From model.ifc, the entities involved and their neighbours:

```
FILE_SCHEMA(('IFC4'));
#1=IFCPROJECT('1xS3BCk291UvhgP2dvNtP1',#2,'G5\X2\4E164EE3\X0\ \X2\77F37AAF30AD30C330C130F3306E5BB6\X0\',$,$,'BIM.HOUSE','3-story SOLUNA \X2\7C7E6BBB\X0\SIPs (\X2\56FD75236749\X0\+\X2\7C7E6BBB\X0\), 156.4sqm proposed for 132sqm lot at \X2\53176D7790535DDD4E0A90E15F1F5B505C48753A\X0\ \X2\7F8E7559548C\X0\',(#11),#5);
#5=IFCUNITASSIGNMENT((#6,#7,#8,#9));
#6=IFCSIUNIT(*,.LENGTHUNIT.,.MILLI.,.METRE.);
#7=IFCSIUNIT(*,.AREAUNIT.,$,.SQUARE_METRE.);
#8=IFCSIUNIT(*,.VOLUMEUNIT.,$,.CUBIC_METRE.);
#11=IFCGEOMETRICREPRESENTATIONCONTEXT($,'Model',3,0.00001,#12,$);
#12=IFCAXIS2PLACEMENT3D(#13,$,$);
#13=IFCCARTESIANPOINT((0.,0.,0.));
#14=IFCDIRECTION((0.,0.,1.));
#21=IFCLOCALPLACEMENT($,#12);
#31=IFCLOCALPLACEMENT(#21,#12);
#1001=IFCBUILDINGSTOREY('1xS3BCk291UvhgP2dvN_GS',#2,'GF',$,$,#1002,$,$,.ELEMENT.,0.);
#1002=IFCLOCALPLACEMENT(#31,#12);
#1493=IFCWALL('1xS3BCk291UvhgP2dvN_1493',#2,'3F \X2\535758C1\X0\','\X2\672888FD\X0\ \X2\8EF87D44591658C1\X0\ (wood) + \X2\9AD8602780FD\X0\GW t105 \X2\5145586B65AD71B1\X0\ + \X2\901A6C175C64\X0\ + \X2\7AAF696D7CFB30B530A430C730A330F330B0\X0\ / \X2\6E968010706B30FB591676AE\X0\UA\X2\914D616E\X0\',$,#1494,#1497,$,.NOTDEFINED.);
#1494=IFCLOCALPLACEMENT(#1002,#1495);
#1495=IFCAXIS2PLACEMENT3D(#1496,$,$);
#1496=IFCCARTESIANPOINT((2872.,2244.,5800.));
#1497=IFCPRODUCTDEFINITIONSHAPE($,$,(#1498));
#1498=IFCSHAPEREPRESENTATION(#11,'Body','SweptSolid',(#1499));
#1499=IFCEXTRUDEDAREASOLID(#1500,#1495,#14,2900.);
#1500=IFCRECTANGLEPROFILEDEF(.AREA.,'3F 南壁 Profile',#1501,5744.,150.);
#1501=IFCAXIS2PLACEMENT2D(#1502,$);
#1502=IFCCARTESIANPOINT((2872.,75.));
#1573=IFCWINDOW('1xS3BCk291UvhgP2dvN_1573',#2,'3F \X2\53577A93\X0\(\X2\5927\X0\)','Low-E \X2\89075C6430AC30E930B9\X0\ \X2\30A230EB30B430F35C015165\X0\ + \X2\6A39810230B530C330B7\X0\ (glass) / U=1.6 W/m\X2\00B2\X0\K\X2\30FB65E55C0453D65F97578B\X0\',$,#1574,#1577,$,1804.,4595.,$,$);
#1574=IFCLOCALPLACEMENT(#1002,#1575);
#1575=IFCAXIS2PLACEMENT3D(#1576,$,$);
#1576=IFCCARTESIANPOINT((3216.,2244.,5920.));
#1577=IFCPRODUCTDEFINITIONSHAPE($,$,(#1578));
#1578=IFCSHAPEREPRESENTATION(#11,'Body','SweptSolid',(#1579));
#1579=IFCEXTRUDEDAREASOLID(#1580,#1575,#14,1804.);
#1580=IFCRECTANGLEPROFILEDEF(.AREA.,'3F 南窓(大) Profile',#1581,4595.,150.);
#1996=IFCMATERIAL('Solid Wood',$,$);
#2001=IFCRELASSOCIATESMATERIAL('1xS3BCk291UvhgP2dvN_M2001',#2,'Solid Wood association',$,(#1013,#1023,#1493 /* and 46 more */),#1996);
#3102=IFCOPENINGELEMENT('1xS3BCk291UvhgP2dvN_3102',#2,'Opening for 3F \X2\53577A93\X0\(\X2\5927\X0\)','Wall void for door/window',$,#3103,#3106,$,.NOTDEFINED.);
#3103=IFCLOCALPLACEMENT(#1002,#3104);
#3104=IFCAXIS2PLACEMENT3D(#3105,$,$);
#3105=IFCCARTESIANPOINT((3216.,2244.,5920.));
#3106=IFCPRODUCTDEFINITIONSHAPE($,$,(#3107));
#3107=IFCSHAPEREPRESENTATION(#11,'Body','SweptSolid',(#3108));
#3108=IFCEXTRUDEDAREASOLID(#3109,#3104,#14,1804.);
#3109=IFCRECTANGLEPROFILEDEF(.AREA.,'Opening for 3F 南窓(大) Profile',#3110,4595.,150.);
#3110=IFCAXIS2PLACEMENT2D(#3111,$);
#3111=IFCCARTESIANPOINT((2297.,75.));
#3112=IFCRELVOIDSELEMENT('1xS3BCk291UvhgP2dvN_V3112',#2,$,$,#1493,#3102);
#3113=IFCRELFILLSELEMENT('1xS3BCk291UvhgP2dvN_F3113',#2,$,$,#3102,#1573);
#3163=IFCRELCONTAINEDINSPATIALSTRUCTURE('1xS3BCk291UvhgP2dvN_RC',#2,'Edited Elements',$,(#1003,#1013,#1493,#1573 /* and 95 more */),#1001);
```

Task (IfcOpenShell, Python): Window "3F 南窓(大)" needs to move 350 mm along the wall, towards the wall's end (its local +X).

```python
import ifcopenshell
import ifcopenshell.api.geometry
import ifcopenshell.util.placement

model = ifcopenshell.open("model.ifc")

window = model.by_guid("1xS3BCk291UvhgP2dvN_1573")
opening = window.FillsVoids[0].RelatingOpeningElement
wall = opening.VoidsElements[0].RelatingBuildingElement

wall_matrix = ifcopenshell.util.placement.get_local_placement(wall.ObjectPlacement)
shift = wall_matrix[:3, 0] * 350.0
before = ifcopenshell.util.placement.get_local_placement(window.ObjectPlacement)[:3, 3].copy()

# The window is not placed relative to its opening, so move both.
for product in (opening, window):
    matrix = ifcopenshell.util.placement.get_local_placement(product.ObjectPlacement)
    matrix[:3, 3] += shift
    ifcopenshell.api.geometry.edit_object_placement(model, product=product, matrix=matrix, is_si=False)

after = ifcopenshell.util.placement.get_local_placement(window.ObjectPlacement)[:3, 3]
print("window moved by", (after - before).round(3) + 0.0)

model.write("model_updated.ifc")
```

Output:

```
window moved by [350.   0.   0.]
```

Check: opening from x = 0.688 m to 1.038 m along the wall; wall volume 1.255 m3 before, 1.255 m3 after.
